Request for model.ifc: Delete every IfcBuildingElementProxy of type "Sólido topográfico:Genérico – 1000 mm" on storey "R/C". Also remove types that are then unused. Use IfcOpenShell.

First a look at what the model holds.

```python
import ifcopenshell
import ifcopenshell.util.element

model = ifcopenshell.open("model.ifc")
print(model.schema)
storey = next(s for s in model.by_type("IfcBuildingStorey") if s.Name == "R/C")
proxies = [e for e in ifcopenshell.util.element.get_decomposition(storey) if e.is_a("IfcBuildingElementProxy")]
seen = {}
for e in proxies:
    element_type = ifcopenshell.util.element.get_type(e)
    name = element_type.Name if element_type not in (None, e) else None
    seen[name] = seen.get(name, 0) + 1
for name, count in sorted(seen.items(), key=str):
    print(count, "x", name)
```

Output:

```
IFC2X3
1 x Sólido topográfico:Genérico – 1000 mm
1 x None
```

```python
import ifcopenshell
import ifcopenshell.api.root
import ifcopenshell.util.element

model = ifcopenshell.open("model.ifc")

storey = next(s for s in model.by_type("IfcBuildingStorey") if s.Name == "R/C")
proxies = [e for e in ifcopenshell.util.element.get_decomposition(storey) if e.is_a("IfcBuildingElementProxy")]
targets = [e for e in proxies if (t := ifcopenshell.util.element.get_type(e)) not in (None, e) and t.Name == 'Sólido topográfico:Genérico – 1000\xa0mm']
types = {ifcopenshell.util.element.get_type(e) for e in targets} - {None, *targets}

for e in targets:
    ifcopenshell.api.root.remove_product(model, product=e)
print(len(targets), "removed")

unused = [t for t in types if not ifcopenshell.util.element.get_types(t)]
for t in unused:
    ifcopenshell.api.root.remove_product(model, product=t)
print(len(unused), "unused types removed")

model.write("model-out.ifc")
```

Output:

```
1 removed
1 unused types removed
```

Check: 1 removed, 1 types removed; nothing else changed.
